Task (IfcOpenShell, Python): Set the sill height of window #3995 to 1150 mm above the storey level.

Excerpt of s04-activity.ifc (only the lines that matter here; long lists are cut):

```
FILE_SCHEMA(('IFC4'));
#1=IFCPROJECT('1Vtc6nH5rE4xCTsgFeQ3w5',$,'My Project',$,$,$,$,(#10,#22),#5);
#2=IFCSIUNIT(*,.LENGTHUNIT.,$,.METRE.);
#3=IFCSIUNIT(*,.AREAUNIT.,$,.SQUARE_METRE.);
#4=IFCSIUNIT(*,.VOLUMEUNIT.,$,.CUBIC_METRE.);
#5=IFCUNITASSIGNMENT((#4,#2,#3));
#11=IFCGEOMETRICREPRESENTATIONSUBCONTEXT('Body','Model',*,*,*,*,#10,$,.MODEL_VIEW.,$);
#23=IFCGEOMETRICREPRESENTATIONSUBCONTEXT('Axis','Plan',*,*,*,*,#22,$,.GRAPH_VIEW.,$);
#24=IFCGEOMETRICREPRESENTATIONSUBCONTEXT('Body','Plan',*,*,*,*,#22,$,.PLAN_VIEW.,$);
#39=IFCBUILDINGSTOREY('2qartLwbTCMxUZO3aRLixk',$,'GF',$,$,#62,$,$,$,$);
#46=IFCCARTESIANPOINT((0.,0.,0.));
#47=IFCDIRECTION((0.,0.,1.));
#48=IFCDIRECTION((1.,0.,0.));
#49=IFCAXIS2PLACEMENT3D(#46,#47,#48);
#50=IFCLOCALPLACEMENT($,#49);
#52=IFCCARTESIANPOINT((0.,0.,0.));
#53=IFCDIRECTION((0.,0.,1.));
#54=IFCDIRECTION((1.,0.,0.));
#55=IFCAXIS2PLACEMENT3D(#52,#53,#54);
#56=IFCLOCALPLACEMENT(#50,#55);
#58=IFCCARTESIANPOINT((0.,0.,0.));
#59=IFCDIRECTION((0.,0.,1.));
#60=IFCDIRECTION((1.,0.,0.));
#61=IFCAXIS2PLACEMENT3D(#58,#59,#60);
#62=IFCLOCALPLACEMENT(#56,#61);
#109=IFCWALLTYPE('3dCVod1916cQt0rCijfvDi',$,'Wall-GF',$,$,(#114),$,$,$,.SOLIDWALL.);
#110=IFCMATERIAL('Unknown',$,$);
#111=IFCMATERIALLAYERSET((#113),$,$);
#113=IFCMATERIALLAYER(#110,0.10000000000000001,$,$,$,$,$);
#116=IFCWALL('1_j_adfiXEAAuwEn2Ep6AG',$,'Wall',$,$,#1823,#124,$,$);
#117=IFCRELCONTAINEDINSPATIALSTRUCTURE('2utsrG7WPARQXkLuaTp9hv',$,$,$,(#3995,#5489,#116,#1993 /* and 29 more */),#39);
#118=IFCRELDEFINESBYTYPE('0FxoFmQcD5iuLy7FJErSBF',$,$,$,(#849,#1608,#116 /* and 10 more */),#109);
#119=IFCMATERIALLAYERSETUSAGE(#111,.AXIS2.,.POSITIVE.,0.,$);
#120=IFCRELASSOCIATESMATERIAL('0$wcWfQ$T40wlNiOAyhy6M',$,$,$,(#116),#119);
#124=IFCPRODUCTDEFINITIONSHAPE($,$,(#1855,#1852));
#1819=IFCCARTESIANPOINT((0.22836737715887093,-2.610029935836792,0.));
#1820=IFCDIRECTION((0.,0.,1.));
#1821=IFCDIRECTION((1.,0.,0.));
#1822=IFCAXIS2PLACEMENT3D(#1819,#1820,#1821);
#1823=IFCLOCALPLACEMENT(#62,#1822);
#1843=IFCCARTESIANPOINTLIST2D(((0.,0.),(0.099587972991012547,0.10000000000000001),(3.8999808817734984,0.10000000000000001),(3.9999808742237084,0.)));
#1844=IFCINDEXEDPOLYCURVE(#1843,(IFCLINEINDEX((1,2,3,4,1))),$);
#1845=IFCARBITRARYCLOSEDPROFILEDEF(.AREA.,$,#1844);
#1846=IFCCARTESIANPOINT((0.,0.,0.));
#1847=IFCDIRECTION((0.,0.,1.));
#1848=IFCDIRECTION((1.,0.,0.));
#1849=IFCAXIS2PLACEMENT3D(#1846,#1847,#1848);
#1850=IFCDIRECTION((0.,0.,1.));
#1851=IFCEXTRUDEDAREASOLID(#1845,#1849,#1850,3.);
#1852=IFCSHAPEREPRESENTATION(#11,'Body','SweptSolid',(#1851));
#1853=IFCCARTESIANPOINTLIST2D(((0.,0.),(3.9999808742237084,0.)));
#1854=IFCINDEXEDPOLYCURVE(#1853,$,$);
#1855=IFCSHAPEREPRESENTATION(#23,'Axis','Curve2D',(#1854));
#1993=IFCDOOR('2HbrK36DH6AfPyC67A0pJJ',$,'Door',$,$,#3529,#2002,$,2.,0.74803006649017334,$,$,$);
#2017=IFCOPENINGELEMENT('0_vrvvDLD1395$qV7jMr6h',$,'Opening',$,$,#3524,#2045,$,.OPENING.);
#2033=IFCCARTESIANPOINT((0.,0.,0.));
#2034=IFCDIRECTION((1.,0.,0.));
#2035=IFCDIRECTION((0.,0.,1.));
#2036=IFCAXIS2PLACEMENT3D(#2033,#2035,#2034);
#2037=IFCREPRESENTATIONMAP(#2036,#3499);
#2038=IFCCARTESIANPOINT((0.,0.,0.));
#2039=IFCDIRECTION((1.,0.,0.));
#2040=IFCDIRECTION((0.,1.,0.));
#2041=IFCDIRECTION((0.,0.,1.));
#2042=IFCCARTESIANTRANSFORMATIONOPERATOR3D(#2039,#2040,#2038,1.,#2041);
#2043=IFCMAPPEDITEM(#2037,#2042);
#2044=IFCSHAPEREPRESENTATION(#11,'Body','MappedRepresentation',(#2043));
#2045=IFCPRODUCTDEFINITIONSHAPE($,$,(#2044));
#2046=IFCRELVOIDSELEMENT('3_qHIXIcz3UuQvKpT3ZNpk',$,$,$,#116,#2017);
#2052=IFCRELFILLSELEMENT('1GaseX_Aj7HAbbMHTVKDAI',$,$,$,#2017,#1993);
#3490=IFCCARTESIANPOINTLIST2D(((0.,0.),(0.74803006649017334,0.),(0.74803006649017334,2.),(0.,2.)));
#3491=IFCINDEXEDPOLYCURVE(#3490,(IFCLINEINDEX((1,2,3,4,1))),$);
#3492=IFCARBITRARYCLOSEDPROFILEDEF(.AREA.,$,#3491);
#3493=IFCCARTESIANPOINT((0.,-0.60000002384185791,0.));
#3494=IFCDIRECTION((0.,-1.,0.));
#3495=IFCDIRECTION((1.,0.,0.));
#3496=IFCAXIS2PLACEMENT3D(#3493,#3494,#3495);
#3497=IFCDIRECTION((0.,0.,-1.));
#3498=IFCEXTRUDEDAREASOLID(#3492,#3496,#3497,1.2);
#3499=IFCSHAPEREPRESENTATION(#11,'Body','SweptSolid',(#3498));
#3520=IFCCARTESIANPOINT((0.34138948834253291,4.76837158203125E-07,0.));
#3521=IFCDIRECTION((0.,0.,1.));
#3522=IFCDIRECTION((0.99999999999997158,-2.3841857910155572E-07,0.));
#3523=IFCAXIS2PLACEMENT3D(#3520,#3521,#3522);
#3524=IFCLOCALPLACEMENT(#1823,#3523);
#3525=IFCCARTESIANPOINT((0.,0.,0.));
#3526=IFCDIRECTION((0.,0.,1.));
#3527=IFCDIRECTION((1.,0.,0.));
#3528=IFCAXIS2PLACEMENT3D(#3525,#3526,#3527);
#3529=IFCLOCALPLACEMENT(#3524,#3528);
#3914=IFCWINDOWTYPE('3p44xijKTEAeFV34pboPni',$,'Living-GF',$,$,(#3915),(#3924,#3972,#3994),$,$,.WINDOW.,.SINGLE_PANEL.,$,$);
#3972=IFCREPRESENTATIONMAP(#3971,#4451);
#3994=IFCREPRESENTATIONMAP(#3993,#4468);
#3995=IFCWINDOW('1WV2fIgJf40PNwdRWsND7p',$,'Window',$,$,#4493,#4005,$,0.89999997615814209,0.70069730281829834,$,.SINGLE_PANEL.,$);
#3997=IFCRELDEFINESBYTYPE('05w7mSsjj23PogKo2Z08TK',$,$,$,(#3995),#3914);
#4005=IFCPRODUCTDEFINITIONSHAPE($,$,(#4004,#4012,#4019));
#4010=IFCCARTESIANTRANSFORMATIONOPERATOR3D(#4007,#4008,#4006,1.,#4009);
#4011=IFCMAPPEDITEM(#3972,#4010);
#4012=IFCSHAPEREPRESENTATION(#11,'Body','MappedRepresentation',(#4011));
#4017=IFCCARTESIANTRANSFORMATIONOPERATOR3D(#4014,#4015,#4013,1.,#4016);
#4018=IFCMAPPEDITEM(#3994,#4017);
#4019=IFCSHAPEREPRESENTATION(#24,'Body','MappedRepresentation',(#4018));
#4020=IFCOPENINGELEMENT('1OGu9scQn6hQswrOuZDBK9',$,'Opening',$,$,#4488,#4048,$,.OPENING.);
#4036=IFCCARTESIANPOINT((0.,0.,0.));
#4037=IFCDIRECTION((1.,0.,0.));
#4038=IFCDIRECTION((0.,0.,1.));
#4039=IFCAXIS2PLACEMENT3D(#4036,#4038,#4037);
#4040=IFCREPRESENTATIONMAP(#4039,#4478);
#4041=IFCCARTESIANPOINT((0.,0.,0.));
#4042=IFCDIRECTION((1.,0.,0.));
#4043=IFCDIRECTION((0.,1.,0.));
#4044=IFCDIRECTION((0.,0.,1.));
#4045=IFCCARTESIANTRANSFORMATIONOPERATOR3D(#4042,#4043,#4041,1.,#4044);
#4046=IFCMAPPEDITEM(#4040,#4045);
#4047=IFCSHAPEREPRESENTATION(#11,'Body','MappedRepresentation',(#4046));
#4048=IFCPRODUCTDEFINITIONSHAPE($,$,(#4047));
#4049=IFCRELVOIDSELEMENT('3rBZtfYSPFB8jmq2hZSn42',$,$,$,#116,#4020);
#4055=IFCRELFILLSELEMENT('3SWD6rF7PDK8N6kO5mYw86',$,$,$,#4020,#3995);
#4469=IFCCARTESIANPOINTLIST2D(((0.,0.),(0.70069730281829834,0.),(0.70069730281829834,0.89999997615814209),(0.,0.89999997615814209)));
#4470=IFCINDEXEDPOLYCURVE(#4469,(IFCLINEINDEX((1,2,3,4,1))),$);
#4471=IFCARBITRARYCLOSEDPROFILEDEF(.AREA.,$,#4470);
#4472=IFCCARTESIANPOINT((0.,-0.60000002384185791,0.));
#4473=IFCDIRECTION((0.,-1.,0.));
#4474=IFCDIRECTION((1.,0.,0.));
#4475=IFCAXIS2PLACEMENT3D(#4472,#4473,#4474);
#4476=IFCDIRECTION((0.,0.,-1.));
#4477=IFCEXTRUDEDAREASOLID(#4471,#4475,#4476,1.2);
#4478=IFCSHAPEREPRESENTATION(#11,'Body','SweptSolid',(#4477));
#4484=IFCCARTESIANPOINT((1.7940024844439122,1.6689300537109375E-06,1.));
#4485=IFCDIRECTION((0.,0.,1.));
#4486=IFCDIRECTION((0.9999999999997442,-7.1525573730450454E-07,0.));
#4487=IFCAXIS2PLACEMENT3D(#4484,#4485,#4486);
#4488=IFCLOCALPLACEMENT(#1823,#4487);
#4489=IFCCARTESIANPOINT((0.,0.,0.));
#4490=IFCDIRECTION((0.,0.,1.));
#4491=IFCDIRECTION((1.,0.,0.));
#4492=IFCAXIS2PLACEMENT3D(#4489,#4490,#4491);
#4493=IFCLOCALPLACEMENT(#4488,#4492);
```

```python
import numpy as np
import ifcopenshell
import ifcopenshell.api.geometry
import ifcopenshell.geom
import ifcopenshell.util.element
import ifcopenshell.util.placement
import ifcopenshell.util.shape
import ifcopenshell.util.unit

model = ifcopenshell.open("s04-activity.ifc")
unit_scale = ifcopenshell.util.unit.calculate_unit_scale(model)

window = model.by_id(3995)
opening = window.FillsVoids[0].RelatingOpeningElement
storey = ifcopenshell.util.element.get_container(window, ifc_class="IfcBuildingStorey")
level = ifcopenshell.util.placement.get_local_placement(storey.ObjectPlacement)[2, 3]

# The opening's origin need not be at the sill, so measure its lowest point.
shape = ifcopenshell.geom.create_shape(ifcopenshell.geom.settings(), opening)
bottom = ifcopenshell.util.shape.get_shape_bottom_elevation(shape, shape.geometry) / unit_scale
dz = level + 1.15 - bottom

shift = np.array([0.0, 0.0, dz])
# The window is placed relative to its opening, so it follows when the opening moves.
matrix = ifcopenshell.util.placement.get_local_placement(opening.ObjectPlacement)
matrix[:3, 3] += shift
ifcopenshell.api.geometry.edit_object_placement(
    model, product=opening, matrix=matrix, is_si=False, should_transform_children=True
)

print(f"moved by {dz * unit_scale:+.3f} m")

model.write("s04-activity_v2.ifc")
```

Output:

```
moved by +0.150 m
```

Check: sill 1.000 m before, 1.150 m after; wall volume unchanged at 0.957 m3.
